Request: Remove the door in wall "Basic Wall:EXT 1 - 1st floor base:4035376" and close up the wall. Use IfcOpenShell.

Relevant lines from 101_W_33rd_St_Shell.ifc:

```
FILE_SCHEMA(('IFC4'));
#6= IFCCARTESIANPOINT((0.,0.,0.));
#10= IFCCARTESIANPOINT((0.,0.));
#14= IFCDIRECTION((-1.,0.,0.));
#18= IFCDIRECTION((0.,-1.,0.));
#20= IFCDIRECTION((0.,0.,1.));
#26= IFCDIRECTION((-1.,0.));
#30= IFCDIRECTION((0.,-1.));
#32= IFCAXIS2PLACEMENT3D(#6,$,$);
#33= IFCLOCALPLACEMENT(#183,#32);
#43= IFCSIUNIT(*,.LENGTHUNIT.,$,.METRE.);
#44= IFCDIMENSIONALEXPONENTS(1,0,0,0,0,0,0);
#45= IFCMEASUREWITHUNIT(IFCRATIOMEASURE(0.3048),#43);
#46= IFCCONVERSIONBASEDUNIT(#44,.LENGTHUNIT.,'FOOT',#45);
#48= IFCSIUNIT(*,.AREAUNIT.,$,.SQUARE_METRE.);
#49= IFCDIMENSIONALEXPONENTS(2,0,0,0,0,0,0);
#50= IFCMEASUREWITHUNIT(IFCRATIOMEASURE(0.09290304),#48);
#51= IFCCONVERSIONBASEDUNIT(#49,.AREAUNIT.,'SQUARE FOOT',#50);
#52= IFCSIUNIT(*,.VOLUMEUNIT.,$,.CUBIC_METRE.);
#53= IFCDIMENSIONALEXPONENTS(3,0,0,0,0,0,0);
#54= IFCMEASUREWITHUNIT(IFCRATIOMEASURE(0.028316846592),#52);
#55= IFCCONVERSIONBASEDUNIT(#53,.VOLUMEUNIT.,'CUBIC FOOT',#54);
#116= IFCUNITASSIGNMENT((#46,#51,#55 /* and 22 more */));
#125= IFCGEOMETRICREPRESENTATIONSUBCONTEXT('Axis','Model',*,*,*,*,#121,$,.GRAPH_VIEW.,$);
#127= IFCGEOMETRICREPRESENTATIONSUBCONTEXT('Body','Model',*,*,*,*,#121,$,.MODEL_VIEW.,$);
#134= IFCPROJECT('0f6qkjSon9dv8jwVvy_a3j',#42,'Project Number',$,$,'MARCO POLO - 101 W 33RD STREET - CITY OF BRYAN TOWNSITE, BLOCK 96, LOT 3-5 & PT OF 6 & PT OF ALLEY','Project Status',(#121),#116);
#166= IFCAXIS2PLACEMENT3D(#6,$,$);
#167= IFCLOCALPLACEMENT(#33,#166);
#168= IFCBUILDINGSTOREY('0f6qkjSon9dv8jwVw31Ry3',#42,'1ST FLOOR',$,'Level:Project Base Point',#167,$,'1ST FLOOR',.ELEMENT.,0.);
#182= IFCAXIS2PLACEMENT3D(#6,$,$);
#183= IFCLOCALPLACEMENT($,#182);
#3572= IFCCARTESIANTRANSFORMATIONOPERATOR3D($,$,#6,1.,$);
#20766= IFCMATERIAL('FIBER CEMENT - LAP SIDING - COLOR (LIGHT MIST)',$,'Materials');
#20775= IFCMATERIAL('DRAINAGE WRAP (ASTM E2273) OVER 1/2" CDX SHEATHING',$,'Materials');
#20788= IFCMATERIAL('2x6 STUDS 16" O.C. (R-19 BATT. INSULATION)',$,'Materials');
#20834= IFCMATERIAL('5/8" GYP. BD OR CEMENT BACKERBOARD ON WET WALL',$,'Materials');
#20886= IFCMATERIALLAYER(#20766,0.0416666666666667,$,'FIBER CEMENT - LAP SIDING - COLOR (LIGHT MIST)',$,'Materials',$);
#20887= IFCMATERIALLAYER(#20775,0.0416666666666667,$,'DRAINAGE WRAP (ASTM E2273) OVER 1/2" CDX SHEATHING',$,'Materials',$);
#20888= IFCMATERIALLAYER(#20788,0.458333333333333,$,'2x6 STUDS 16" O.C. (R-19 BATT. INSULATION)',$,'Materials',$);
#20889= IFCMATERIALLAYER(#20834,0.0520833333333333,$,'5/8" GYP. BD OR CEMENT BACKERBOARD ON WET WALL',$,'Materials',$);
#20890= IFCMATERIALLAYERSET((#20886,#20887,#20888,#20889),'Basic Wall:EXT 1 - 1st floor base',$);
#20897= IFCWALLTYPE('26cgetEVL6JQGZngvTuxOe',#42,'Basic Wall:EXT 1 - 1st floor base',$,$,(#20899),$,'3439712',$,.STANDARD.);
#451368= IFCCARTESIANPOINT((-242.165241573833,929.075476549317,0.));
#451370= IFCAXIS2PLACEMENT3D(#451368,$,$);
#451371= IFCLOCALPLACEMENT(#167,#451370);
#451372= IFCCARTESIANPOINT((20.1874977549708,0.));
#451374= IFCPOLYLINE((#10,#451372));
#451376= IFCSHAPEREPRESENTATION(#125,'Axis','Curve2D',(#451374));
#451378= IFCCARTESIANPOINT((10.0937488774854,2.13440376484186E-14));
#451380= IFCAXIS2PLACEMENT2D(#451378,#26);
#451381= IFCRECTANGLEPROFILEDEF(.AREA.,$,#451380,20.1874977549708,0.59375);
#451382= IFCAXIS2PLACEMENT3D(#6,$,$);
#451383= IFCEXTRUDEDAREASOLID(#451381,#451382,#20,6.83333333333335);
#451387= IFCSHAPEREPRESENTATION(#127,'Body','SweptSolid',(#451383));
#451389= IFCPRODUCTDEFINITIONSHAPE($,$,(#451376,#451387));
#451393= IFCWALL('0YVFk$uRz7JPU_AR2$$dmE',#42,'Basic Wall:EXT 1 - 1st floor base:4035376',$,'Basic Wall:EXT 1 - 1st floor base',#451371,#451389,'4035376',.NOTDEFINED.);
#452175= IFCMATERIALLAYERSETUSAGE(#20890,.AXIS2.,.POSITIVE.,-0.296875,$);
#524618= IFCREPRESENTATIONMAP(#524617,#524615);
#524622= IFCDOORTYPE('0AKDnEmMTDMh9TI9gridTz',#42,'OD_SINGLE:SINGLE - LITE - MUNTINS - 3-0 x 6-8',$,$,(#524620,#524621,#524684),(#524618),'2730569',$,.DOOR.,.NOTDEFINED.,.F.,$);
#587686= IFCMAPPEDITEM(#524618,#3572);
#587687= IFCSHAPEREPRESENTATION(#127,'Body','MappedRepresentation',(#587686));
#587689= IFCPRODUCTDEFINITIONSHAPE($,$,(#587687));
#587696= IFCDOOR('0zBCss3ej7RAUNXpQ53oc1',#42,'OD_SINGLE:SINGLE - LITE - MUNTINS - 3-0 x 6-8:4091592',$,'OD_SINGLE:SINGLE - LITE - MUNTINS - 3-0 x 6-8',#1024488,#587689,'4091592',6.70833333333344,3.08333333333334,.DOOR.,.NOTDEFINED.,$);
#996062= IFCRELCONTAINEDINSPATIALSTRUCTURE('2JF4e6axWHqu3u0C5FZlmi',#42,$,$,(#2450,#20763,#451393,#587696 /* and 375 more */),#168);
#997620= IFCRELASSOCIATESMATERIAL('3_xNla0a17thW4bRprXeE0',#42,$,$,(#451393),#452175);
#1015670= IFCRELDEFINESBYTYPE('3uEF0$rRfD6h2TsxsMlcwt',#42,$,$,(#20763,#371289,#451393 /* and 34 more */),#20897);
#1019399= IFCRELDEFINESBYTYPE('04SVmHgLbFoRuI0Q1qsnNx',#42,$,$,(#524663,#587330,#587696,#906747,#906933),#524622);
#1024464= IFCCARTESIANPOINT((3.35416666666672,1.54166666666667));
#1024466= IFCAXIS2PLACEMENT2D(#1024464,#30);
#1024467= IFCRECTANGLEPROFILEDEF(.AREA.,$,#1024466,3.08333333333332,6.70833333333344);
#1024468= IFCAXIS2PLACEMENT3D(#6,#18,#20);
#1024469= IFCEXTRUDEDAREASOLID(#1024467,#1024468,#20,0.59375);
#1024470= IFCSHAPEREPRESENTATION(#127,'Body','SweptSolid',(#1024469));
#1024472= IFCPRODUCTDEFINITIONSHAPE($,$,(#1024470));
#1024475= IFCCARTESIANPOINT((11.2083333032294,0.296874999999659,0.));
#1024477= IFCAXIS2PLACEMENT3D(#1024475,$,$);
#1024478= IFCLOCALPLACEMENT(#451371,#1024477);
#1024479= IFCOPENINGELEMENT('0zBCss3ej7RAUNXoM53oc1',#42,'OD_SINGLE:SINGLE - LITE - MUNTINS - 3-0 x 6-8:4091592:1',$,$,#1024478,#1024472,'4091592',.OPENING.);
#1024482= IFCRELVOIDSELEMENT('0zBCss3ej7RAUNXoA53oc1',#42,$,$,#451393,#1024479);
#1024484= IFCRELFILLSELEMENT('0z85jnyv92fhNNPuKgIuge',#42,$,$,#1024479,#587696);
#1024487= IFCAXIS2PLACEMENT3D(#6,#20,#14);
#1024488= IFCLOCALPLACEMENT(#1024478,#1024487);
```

```python
import ifcopenshell
import ifcopenshell.api.feature
import ifcopenshell.api.root
import ifcopenshell.geom
import ifcopenshell.util.shape

model = ifcopenshell.open("101_W_33rd_St_Shell.ifc")
settings = ifcopenshell.geom.settings()


def volume(element):
    """Net volume in cubic metres, openings subtracted."""
    shape = ifcopenshell.geom.create_shape(settings, element)
    return ifcopenshell.util.shape.get_volume(shape.geometry)


door = model.by_id(587696)
opening = door.FillsVoids[0].RelatingOpeningElement
wall = opening.VoidsElements[0].RelatingBuildingElement
before = volume(wall)

ifcopenshell.api.root.remove_product(model, product=door)
ifcopenshell.api.feature.remove_feature(model, feature=opening)

after = volume(wall)

print(f"wall volume {before:.3f} -> {after:.3f} m3")

model.write("101_W_33rd_St_Shell-out.ifc")
```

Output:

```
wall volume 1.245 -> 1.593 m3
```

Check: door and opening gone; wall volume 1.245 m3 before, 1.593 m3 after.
